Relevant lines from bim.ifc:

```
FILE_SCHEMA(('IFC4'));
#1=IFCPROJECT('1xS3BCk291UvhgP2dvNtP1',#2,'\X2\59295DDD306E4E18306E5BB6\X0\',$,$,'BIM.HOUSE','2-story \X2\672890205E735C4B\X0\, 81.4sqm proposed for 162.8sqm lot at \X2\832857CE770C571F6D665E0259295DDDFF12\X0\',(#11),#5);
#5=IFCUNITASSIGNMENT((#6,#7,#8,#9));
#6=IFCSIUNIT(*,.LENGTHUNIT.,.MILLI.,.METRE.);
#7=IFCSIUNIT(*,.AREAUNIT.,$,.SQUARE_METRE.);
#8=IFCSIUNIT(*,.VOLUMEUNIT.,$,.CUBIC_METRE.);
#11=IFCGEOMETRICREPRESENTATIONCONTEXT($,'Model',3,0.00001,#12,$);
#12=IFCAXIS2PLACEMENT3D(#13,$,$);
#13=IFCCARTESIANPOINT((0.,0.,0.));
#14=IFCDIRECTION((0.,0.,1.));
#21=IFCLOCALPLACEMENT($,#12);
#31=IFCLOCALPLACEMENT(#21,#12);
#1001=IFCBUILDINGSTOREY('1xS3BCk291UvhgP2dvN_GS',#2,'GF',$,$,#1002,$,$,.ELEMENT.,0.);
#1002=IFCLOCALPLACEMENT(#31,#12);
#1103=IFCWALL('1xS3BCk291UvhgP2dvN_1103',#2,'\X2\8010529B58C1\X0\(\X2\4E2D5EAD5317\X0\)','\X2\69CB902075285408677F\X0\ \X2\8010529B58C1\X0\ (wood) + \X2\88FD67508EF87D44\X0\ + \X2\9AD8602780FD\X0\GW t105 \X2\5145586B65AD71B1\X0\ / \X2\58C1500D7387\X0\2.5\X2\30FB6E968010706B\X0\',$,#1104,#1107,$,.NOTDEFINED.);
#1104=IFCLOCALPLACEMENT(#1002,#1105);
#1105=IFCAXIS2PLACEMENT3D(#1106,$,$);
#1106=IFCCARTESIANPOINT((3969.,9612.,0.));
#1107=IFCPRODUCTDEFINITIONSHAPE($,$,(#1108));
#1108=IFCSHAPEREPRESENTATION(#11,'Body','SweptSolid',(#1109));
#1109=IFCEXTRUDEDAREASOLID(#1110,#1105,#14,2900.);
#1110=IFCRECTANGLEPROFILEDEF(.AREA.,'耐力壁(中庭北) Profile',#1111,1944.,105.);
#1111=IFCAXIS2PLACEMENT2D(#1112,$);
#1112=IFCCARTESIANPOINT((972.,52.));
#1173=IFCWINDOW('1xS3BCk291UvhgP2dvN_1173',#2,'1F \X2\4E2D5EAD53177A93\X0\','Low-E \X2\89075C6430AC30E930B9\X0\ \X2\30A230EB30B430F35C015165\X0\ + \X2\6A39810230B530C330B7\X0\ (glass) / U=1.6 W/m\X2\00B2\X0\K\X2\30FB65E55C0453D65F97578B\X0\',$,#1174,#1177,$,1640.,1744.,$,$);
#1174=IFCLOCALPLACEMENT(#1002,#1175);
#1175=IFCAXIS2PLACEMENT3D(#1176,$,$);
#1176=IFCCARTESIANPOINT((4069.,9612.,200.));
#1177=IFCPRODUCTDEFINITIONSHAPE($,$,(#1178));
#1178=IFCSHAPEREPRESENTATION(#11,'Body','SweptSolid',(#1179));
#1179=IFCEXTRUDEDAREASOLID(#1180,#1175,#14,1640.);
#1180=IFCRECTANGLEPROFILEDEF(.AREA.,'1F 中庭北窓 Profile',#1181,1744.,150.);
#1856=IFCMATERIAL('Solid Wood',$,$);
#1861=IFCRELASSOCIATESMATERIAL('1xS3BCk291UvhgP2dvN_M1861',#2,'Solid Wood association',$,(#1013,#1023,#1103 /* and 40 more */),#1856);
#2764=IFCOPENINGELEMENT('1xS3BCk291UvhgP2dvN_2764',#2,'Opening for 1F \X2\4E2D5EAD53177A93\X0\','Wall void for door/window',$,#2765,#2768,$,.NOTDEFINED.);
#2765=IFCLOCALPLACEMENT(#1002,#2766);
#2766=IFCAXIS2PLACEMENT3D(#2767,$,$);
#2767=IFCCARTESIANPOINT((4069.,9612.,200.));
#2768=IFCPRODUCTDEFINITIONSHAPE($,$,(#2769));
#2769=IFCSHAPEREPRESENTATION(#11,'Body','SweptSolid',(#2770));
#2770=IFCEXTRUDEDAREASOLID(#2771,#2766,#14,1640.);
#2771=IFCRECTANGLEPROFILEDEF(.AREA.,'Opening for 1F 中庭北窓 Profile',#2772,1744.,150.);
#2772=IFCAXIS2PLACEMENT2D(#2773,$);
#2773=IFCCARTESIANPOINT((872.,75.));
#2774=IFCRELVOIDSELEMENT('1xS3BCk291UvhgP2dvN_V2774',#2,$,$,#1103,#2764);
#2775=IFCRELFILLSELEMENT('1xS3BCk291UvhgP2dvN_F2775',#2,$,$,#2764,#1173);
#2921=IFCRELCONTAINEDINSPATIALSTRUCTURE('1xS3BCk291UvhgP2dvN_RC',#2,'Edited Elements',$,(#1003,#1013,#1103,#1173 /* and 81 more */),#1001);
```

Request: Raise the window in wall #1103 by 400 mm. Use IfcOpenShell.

```python
import numpy as np
import ifcopenshell
import ifcopenshell.api.geometry
import ifcopenshell.util.placement
import ifcopenshell.util.unit

model = ifcopenshell.open("bim.ifc")
unit_scale = ifcopenshell.util.unit.calculate_unit_scale(model)

window = model.by_guid("1xS3BCk291UvhgP2dvN_1173")
opening = window.FillsVoids[0].RelatingOpeningElement
dz = 0.4 / unit_scale

shift = np.array([0.0, 0.0, dz])
# The window is not placed relative to its opening, so move both.
for product in (opening, window):
    matrix = ifcopenshell.util.placement.get_local_placement(product.ObjectPlacement)
    matrix[:3, 3] += shift
    ifcopenshell.api.geometry.edit_object_placement(model, product=product, matrix=matrix, is_si=False)

print(f"moved by {dz * unit_scale:+.3f} m")

model.write("bim_v2.ifc")
```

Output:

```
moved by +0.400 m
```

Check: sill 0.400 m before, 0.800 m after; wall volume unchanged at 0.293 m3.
